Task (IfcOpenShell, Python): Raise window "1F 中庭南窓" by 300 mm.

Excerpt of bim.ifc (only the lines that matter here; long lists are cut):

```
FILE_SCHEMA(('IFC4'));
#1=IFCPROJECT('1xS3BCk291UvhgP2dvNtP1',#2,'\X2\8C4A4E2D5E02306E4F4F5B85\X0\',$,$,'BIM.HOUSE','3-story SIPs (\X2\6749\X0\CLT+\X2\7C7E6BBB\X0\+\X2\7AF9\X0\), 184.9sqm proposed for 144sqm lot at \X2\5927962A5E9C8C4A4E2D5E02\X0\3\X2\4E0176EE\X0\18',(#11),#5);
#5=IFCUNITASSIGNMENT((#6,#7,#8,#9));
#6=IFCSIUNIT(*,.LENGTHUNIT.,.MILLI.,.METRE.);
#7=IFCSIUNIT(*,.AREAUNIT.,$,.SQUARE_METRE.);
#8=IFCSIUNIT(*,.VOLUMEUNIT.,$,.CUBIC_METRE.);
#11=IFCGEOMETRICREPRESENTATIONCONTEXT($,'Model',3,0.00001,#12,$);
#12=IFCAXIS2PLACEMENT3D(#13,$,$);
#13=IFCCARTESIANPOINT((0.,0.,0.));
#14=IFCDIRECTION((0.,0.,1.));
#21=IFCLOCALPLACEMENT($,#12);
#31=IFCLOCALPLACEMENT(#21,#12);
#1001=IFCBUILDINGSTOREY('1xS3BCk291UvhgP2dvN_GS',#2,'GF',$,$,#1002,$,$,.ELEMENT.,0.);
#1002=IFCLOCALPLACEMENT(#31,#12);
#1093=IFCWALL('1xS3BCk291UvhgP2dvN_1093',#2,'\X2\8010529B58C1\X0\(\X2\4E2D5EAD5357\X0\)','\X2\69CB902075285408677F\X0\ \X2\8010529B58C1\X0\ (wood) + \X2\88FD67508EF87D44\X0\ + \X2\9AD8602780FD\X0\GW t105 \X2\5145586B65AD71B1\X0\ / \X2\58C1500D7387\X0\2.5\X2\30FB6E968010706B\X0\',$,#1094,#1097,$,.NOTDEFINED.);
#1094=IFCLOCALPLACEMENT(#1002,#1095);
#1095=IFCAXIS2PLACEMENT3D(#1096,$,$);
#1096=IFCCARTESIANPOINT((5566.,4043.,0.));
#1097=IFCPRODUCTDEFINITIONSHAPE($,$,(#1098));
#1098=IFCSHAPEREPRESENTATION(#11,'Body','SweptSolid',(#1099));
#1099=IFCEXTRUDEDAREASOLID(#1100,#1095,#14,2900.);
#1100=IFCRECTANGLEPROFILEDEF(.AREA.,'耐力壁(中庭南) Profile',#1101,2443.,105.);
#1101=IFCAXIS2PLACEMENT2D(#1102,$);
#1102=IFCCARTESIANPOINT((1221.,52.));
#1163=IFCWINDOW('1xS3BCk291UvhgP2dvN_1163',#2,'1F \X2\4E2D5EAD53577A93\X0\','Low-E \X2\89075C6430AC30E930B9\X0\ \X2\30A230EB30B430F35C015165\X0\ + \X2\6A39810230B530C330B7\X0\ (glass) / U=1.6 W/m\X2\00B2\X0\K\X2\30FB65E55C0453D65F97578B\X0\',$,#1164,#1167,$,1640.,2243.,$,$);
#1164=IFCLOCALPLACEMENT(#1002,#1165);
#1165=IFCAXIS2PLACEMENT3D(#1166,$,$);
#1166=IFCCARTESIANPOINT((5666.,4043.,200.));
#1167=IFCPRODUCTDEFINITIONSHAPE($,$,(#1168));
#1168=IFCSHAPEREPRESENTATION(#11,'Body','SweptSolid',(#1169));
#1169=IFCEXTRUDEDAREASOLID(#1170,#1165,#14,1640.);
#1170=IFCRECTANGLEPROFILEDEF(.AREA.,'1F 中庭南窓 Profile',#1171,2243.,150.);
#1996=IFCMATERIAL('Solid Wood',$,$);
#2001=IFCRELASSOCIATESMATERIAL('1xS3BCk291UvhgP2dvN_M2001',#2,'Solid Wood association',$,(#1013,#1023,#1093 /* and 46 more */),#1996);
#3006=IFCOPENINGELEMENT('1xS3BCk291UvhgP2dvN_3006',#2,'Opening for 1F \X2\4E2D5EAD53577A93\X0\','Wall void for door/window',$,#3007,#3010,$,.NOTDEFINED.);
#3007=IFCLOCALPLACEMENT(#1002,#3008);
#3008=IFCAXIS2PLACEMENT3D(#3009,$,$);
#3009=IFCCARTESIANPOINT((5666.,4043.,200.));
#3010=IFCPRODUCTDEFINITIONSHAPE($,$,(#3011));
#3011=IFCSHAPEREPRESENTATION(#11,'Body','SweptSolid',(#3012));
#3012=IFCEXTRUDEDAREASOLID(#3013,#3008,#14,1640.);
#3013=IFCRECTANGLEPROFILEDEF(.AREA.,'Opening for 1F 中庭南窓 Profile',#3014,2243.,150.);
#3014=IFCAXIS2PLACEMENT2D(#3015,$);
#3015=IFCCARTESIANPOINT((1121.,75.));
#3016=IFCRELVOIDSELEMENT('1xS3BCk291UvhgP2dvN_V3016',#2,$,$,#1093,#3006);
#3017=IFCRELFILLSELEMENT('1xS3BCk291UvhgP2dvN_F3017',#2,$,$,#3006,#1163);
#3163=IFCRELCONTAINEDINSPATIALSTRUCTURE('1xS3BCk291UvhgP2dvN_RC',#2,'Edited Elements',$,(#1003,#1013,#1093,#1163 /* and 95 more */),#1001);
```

```python
import numpy as np
import ifcopenshell
import ifcopenshell.api.geometry
import ifcopenshell.util.placement
import ifcopenshell.util.unit

model = ifcopenshell.open("bim.ifc")
unit_scale = ifcopenshell.util.unit.calculate_unit_scale(model)

window = model.by_id(1163)
opening = window.FillsVoids[0].RelatingOpeningElement
dz = 0.3 / unit_scale

shift = np.array([0.0, 0.0, dz])
# The window is not placed relative to its opening, so move both.
for product in (opening, window):
    matrix = ifcopenshell.util.placement.get_local_placement(product.ObjectPlacement)
    matrix[:3, 3] += shift
    ifcopenshell.api.geometry.edit_object_placement(model, product=product, matrix=matrix, is_si=False)

print(f"moved by {dz * unit_scale:+.3f} m")

model.write("bim_edited.ifc")
```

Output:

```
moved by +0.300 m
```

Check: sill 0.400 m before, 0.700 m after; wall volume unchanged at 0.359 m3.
